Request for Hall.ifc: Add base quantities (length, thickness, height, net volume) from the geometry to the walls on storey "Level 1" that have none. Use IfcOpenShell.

First a look at what the model holds.

```python
import ifcopenshell
import ifcopenshell.util.element
import ifcopenshell.util.unit

model = ifcopenshell.open("Hall.ifc")
print(model.schema)
for unit_type in ("LENGTHUNIT", "AREAUNIT", "VOLUMEUNIT"):
    print(unit_type, ifcopenshell.util.unit.calculate_unit_scale(model, unit_type))
storey = next(s for s in model.by_type("IfcBuildingStorey") if s.Name == "Level 1")
walls = [e for e in ifcopenshell.util.element.get_decomposition(storey) if e.is_a("IfcWall")]
for e in sorted(walls, key=lambda e: e.id()):
    print(e.id(), e.is_a(), e.Name, list(ifcopenshell.util.element.get_psets(e, qtos_only=True)), sep=" | ")
```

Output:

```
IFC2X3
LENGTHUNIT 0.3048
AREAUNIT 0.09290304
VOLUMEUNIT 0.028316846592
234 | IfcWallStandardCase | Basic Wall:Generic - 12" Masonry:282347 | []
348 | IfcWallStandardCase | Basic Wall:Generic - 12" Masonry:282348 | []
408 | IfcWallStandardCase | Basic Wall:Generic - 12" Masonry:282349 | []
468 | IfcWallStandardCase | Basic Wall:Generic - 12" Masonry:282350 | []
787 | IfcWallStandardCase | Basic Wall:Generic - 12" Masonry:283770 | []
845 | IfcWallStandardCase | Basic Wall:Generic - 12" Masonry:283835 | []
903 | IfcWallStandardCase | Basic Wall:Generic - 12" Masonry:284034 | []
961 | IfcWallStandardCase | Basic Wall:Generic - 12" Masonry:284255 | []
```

```python
import ifcopenshell
import ifcopenshell.api.pset
import ifcopenshell.geom
import ifcopenshell.util.element
import ifcopenshell.util.shape
import ifcopenshell.util.unit

model = ifcopenshell.open("Hall.ifc")
unit_scale = ifcopenshell.util.unit.calculate_unit_scale(model)
volume_scale = ifcopenshell.util.unit.calculate_unit_scale(model, "VOLUMEUNIT")
settings = ifcopenshell.geom.settings()

storey = next(s for s in model.by_type("IfcBuildingStorey") if s.Name == "Level 1")
walls = [e for e in ifcopenshell.util.element.get_decomposition(storey) if e.is_a("IfcWall")]

for e in sorted(walls, key=lambda e: e.id()):
    if ifcopenshell.util.element.get_psets(e, qtos_only=True, should_inherit=False):
        continue
    # Geometry comes back in metres, in the element's own axes.
    shape = ifcopenshell.geom.create_shape(settings, e)
    values = {
        "Length": ifcopenshell.util.shape.get_x(shape.geometry) / unit_scale,
        "Width": ifcopenshell.util.shape.get_y(shape.geometry) / unit_scale,
        "Height": ifcopenshell.util.shape.get_z(shape.geometry) / unit_scale,
        "NetVolume": ifcopenshell.util.shape.get_volume(shape.geometry) / volume_scale,
    }
    qto = ifcopenshell.api.pset.add_qto(model, product=e, name="BaseQuantities")
    ifcopenshell.api.pset.edit_qto(model, qto=qto, properties=values)
    print(e.id(), {k: round(v, 3) for k, v in values.items()})

model.write("Hall_updated.ifc")
```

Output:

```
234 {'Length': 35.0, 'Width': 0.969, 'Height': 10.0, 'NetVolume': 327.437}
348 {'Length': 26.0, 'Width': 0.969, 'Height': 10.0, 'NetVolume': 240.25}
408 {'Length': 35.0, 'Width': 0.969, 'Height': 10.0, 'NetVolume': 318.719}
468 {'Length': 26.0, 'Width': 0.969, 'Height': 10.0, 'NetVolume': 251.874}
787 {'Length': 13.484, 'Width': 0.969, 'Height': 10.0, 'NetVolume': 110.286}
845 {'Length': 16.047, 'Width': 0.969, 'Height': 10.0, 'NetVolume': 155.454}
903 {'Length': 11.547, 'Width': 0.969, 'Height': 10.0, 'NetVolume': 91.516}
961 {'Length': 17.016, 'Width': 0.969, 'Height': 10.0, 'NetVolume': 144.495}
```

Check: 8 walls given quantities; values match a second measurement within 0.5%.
